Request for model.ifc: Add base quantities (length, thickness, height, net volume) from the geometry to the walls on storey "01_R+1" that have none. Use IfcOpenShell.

First a look at what the model holds.

```python
import ifcopenshell
import ifcopenshell.util.element
import ifcopenshell.util.unit

model = ifcopenshell.open("model.ifc")
print(model.schema)
for unit_type in ("LENGTHUNIT", "AREAUNIT", "VOLUMEUNIT"):
    print(unit_type, ifcopenshell.util.unit.calculate_unit_scale(model, unit_type))
storey = next(s for s in model.by_type("IfcBuildingStorey") if s.Name == "01_R+1")
walls = [e for e in ifcopenshell.util.element.get_decomposition(storey) if e.is_a("IfcWall")]
for e in sorted(walls, key=lambda e: e.id()):
    print(e.id(), e.is_a(), e.Name, list(ifcopenshell.util.element.get_psets(e, qtos_only=True)), sep=" | ")
```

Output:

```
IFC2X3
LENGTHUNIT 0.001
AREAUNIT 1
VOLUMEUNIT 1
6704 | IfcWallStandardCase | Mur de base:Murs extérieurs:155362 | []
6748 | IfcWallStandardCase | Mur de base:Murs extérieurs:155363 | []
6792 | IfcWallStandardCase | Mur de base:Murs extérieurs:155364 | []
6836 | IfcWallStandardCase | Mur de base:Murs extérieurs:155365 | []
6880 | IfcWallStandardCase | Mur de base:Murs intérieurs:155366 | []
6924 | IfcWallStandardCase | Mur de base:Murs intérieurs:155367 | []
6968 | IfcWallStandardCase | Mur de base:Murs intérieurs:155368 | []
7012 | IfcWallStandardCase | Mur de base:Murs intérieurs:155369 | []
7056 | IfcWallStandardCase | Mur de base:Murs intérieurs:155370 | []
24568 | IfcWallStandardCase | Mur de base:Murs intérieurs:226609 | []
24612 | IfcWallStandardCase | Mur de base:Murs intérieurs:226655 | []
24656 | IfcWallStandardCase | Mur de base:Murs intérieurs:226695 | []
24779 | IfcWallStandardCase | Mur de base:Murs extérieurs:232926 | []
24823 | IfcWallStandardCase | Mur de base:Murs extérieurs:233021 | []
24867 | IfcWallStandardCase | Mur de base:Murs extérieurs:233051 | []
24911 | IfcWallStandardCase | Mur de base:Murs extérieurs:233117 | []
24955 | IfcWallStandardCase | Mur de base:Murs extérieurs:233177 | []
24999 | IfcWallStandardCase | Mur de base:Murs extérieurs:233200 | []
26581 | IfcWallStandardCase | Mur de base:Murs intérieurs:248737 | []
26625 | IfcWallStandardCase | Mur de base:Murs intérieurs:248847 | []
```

```python
import ifcopenshell
import ifcopenshell.api.pset
import ifcopenshell.geom
import ifcopenshell.util.element
import ifcopenshell.util.shape
import ifcopenshell.util.unit

model = ifcopenshell.open("model.ifc")
unit_scale = ifcopenshell.util.unit.calculate_unit_scale(model)
volume_scale = ifcopenshell.util.unit.calculate_unit_scale(model, "VOLUMEUNIT")
settings = ifcopenshell.geom.settings()

storey = next(s for s in model.by_type("IfcBuildingStorey") if s.Name == "01_R+1")
walls = [e for e in ifcopenshell.util.element.get_decomposition(storey) if e.is_a("IfcWall")]

for e in sorted(walls, key=lambda e: e.id()):
    if ifcopenshell.util.element.get_psets(e, qtos_only=True, should_inherit=False):
        continue
    # Geometry comes back in metres, in the element's own axes.
    shape = ifcopenshell.geom.create_shape(settings, e)
    values = {
        "Length": ifcopenshell.util.shape.get_x(shape.geometry) / unit_scale,
        "Width": ifcopenshell.util.shape.get_y(shape.geometry) / unit_scale,
        "Height": ifcopenshell.util.shape.get_z(shape.geometry) / unit_scale,
        "NetVolume": ifcopenshell.util.shape.get_volume(shape.geometry) / volume_scale,
    }
    qto = ifcopenshell.api.pset.add_qto(model, product=e, name="BaseQuantities")
    ifcopenshell.api.pset.edit_qto(model, qto=qto, properties=values)
    print(e.id(), {k: round(v, 3) for k, v in values.items()})

model.write("model-out.ifc")
```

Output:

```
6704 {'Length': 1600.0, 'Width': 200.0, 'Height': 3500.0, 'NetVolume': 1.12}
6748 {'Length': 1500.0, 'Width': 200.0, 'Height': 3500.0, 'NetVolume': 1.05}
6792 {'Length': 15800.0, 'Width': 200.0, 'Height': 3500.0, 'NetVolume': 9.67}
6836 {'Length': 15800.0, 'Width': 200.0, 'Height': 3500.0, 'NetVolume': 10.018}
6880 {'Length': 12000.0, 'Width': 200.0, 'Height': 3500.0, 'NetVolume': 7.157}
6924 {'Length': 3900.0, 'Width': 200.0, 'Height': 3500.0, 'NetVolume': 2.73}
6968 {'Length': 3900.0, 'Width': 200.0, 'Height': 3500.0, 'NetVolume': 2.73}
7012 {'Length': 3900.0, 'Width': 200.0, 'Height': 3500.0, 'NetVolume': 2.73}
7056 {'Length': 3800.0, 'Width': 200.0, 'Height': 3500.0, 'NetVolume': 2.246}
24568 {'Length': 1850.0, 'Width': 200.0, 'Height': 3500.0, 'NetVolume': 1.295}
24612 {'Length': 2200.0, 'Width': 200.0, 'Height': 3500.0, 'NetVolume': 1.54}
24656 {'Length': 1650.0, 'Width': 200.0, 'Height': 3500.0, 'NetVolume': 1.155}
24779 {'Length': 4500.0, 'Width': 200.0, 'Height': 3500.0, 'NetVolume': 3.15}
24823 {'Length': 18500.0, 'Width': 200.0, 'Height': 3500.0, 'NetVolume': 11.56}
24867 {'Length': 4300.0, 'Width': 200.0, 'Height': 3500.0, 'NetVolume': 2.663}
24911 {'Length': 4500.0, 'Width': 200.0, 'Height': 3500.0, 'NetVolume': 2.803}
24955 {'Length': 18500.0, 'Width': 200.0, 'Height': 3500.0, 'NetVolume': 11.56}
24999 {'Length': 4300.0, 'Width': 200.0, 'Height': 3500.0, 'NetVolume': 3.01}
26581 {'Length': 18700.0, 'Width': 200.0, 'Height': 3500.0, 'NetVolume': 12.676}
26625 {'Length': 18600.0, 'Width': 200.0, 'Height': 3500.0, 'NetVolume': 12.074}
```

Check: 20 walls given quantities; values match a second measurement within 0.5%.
